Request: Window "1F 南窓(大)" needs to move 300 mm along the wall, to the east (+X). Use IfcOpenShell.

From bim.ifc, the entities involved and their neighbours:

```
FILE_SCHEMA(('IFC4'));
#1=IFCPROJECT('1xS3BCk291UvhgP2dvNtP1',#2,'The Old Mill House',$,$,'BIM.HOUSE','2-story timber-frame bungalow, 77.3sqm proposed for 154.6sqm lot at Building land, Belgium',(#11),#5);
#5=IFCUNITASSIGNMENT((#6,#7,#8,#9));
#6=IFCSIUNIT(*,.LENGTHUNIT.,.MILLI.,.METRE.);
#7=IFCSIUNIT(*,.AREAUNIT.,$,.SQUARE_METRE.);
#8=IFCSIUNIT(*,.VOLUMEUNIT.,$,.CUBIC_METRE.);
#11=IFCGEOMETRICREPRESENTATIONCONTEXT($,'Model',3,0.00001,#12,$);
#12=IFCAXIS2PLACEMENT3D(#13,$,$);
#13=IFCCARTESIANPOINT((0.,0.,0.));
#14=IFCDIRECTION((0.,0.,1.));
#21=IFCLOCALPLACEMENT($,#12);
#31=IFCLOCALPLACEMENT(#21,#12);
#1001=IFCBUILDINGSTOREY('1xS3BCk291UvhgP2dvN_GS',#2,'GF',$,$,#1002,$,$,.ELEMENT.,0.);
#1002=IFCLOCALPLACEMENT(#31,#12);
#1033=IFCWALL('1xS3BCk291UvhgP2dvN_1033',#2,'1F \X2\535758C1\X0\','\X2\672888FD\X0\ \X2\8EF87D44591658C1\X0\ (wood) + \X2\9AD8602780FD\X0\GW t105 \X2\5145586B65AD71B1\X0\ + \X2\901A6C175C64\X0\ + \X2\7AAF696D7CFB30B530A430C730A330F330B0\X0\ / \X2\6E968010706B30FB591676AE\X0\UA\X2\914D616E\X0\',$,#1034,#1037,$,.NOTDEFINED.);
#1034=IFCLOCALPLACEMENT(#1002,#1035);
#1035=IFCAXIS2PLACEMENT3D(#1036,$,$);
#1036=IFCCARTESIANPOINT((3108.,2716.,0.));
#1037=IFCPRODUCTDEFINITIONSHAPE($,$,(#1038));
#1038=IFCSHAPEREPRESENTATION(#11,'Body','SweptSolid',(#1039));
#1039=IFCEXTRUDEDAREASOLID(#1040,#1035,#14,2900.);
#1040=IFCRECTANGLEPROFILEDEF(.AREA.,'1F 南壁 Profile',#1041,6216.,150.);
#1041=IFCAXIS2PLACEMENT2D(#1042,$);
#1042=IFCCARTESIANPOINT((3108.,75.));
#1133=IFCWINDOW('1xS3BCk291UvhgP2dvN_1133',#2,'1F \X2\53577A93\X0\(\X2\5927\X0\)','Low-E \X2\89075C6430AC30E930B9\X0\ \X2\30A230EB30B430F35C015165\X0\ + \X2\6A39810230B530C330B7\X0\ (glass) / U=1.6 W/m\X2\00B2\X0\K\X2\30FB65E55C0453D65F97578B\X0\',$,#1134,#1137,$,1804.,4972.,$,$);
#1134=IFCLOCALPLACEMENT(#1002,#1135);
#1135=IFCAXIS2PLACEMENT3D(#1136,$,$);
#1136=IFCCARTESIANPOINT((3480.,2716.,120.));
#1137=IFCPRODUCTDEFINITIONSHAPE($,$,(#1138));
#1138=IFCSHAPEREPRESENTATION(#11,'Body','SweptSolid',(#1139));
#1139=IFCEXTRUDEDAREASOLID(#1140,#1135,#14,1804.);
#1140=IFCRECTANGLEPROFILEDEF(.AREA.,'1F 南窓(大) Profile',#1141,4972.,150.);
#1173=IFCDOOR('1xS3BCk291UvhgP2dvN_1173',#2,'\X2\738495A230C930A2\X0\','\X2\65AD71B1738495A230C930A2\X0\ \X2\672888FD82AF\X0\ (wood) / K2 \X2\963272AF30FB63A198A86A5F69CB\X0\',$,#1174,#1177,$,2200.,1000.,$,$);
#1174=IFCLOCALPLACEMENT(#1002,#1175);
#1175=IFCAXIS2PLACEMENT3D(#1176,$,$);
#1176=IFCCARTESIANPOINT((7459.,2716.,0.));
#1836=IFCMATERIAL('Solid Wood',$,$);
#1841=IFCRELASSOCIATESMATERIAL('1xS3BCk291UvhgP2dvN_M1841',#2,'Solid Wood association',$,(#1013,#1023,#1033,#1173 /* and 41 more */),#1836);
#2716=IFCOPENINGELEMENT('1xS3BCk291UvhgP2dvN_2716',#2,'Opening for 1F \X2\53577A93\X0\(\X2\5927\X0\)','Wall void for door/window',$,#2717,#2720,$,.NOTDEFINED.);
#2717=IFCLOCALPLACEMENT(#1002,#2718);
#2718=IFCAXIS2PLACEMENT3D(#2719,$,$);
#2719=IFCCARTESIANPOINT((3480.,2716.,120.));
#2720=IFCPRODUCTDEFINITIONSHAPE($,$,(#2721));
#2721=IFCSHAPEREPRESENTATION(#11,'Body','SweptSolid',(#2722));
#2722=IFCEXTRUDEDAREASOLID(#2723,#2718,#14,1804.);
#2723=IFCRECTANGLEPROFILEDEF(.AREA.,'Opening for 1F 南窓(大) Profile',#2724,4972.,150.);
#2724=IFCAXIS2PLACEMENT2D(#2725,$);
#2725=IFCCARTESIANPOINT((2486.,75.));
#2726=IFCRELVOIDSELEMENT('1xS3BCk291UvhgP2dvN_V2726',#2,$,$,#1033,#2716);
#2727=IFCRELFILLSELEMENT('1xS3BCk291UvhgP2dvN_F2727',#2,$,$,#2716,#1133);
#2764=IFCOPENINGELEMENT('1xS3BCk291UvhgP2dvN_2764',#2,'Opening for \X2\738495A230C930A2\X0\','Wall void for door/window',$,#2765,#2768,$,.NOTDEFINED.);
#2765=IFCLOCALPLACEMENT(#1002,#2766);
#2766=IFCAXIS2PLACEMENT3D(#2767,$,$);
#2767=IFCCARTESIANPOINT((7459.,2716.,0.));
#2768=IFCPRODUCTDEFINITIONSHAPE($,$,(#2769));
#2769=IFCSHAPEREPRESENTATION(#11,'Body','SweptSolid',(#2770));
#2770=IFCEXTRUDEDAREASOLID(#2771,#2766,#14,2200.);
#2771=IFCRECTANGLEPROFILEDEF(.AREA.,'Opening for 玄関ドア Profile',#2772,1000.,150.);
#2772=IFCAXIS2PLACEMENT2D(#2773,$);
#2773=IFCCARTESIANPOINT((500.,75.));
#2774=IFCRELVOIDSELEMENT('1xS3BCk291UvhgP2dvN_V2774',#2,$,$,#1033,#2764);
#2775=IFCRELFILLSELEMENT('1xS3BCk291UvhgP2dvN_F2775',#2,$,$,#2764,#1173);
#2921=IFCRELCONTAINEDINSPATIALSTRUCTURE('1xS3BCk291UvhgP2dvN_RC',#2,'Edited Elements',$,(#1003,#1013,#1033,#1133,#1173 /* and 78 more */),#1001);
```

```python
import ifcopenshell
import ifcopenshell.api.geometry
import ifcopenshell.util.placement
import ifcopenshell.util.unit

model = ifcopenshell.open("bim.ifc")
unit_scale = ifcopenshell.util.unit.calculate_unit_scale(model)

window = model.by_id(1133)
opening = window.FillsVoids[0].RelatingOpeningElement
wall = opening.VoidsElements[0].RelatingBuildingElement

wall_matrix = ifcopenshell.util.placement.get_local_placement(wall.ObjectPlacement)
shift = wall_matrix[:3, 0] * 0.3 / unit_scale
before = ifcopenshell.util.placement.get_local_placement(window.ObjectPlacement)[:3, 3].copy()

# The window is not placed relative to its opening, so move both.
for product in (opening, window):
    matrix = ifcopenshell.util.placement.get_local_placement(product.ObjectPlacement)
    matrix[:3, 3] += shift
    ifcopenshell.api.geometry.edit_object_placement(model, product=product, matrix=matrix, is_si=False)

after = ifcopenshell.util.placement.get_local_placement(window.ObjectPlacement)[:3, 3]
print("window moved by", (after - before).round(3) + 0.0)

model.write("bim_edited.ifc")
```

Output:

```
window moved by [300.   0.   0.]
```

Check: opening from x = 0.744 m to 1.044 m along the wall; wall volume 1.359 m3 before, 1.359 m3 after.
